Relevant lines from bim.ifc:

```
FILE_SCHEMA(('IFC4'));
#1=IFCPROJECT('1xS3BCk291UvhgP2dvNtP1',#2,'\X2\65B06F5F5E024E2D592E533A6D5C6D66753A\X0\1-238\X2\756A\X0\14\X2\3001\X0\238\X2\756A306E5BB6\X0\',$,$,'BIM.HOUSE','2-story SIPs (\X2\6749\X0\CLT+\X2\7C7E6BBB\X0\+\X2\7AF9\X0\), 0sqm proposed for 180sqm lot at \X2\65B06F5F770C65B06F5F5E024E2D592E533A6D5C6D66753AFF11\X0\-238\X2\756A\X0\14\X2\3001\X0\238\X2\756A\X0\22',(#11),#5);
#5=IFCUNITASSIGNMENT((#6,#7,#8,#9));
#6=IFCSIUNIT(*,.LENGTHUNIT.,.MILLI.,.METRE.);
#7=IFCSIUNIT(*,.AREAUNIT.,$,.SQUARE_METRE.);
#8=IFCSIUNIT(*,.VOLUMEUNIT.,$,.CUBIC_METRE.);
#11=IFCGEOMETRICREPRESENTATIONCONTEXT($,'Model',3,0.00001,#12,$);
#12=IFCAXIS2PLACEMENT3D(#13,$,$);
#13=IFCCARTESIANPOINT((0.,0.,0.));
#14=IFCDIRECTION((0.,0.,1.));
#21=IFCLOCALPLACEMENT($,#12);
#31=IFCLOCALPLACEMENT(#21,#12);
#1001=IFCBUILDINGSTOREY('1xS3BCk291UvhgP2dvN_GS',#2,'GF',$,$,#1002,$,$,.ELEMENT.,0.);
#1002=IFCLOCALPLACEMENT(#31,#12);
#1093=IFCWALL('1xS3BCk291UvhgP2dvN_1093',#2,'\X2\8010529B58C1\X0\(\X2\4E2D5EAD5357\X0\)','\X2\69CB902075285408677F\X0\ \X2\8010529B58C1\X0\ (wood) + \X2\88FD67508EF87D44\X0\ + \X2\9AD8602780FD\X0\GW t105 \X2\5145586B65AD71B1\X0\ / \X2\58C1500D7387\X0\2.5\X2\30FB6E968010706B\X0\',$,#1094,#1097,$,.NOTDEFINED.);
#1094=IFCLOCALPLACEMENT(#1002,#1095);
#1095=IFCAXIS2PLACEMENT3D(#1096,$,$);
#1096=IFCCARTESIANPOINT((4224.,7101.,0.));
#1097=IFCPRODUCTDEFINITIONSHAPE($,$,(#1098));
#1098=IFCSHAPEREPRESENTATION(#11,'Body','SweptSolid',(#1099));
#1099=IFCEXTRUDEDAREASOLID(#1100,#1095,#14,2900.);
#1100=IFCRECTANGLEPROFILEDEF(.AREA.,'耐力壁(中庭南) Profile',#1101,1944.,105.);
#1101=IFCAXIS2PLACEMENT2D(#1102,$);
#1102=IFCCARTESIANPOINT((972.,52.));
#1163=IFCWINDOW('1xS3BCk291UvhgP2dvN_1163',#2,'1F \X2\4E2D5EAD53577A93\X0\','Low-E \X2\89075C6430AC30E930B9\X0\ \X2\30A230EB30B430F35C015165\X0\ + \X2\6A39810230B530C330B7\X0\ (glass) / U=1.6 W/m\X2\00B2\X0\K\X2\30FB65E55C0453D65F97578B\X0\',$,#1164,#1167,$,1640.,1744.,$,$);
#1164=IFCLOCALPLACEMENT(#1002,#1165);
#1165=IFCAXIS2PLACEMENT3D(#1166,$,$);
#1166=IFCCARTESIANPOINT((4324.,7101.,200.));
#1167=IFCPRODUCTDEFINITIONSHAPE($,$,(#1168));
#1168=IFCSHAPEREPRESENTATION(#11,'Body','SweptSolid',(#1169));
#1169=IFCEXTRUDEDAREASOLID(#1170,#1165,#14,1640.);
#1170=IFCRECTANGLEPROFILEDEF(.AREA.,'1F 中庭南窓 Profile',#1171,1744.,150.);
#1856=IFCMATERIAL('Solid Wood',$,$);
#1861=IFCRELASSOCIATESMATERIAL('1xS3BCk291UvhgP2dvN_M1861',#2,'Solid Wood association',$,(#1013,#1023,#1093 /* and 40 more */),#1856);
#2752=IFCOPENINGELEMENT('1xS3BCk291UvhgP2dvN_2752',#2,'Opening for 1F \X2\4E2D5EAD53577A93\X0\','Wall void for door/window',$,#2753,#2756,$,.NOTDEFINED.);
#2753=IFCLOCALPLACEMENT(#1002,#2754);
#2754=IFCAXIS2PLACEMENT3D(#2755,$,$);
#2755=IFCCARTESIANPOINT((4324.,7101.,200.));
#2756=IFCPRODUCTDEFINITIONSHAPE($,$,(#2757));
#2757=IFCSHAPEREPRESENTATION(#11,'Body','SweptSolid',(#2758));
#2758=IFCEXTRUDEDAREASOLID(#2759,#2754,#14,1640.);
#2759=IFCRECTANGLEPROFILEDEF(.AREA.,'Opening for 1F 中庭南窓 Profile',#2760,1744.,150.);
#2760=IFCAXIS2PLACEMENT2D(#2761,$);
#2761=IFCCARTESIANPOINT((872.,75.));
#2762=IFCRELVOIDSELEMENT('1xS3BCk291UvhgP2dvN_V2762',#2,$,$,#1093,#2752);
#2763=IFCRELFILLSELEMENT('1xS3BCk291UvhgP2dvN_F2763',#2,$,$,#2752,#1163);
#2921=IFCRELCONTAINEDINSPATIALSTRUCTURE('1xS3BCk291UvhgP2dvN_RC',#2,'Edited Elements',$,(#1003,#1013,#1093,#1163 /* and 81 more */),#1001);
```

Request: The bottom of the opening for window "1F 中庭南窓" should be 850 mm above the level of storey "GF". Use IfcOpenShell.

```python
import numpy as np
import ifcopenshell
import ifcopenshell.api.geometry
import ifcopenshell.geom
import ifcopenshell.util.element
import ifcopenshell.util.placement
import ifcopenshell.util.shape
import ifcopenshell.util.unit

model = ifcopenshell.open("bim.ifc")
unit_scale = ifcopenshell.util.unit.calculate_unit_scale(model)

window = model.by_id(1163)
opening = window.FillsVoids[0].RelatingOpeningElement
storey = ifcopenshell.util.element.get_container(window, ifc_class="IfcBuildingStorey")
level = ifcopenshell.util.placement.get_local_placement(storey.ObjectPlacement)[2, 3]

# The opening's origin need not be at the sill, so measure its lowest point.
shape = ifcopenshell.geom.create_shape(ifcopenshell.geom.settings(), opening)
bottom = ifcopenshell.util.shape.get_shape_bottom_elevation(shape, shape.geometry) / unit_scale
dz = level + 850.0 - bottom

shift = np.array([0.0, 0.0, dz])
# The window is not placed relative to its opening, so move both.
for product in (opening, window):
    matrix = ifcopenshell.util.placement.get_local_placement(product.ObjectPlacement)
    matrix[:3, 3] += shift
    ifcopenshell.api.geometry.edit_object_placement(model, product=product, matrix=matrix, is_si=False)

print(f"moved by {dz * unit_scale:+.3f} m")

model.write("bim_v2.ifc")
```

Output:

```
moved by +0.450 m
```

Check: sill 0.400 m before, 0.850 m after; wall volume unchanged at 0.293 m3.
